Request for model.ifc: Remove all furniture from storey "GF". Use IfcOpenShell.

First a look at what the model holds.

```python
import ifcopenshell
import ifcopenshell.util.element

model = ifcopenshell.open("model.ifc")
print(model.schema)
storey = next(s for s in model.by_type("IfcBuildingStorey") if s.Name == "GF")
furniture = [e for e in ifcopenshell.util.element.get_decomposition(storey) if e.is_a("IfcFurnishingElement")]
seen = {}
for e in furniture:
    element_type = ifcopenshell.util.element.get_type(e)
    name = element_type.Name if element_type not in (None, e) else None
    seen[name] = seen.get(name, 0) + 1
for name, count in sorted(seen.items(), key=str):
    print(count, "x", name)
```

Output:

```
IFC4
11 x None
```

```python
import ifcopenshell
import ifcopenshell.api.root
import ifcopenshell.util.element

model = ifcopenshell.open("model.ifc")

storey = next(s for s in model.by_type("IfcBuildingStorey") if s.Name == "GF")
furniture = [e for e in ifcopenshell.util.element.get_decomposition(storey) if e.is_a("IfcFurnishingElement")]

for e in furniture:
    ifcopenshell.api.root.remove_product(model, product=e)
print(len(furniture), "removed")

model.write("model-out.ifc")
```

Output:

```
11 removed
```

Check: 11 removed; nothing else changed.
